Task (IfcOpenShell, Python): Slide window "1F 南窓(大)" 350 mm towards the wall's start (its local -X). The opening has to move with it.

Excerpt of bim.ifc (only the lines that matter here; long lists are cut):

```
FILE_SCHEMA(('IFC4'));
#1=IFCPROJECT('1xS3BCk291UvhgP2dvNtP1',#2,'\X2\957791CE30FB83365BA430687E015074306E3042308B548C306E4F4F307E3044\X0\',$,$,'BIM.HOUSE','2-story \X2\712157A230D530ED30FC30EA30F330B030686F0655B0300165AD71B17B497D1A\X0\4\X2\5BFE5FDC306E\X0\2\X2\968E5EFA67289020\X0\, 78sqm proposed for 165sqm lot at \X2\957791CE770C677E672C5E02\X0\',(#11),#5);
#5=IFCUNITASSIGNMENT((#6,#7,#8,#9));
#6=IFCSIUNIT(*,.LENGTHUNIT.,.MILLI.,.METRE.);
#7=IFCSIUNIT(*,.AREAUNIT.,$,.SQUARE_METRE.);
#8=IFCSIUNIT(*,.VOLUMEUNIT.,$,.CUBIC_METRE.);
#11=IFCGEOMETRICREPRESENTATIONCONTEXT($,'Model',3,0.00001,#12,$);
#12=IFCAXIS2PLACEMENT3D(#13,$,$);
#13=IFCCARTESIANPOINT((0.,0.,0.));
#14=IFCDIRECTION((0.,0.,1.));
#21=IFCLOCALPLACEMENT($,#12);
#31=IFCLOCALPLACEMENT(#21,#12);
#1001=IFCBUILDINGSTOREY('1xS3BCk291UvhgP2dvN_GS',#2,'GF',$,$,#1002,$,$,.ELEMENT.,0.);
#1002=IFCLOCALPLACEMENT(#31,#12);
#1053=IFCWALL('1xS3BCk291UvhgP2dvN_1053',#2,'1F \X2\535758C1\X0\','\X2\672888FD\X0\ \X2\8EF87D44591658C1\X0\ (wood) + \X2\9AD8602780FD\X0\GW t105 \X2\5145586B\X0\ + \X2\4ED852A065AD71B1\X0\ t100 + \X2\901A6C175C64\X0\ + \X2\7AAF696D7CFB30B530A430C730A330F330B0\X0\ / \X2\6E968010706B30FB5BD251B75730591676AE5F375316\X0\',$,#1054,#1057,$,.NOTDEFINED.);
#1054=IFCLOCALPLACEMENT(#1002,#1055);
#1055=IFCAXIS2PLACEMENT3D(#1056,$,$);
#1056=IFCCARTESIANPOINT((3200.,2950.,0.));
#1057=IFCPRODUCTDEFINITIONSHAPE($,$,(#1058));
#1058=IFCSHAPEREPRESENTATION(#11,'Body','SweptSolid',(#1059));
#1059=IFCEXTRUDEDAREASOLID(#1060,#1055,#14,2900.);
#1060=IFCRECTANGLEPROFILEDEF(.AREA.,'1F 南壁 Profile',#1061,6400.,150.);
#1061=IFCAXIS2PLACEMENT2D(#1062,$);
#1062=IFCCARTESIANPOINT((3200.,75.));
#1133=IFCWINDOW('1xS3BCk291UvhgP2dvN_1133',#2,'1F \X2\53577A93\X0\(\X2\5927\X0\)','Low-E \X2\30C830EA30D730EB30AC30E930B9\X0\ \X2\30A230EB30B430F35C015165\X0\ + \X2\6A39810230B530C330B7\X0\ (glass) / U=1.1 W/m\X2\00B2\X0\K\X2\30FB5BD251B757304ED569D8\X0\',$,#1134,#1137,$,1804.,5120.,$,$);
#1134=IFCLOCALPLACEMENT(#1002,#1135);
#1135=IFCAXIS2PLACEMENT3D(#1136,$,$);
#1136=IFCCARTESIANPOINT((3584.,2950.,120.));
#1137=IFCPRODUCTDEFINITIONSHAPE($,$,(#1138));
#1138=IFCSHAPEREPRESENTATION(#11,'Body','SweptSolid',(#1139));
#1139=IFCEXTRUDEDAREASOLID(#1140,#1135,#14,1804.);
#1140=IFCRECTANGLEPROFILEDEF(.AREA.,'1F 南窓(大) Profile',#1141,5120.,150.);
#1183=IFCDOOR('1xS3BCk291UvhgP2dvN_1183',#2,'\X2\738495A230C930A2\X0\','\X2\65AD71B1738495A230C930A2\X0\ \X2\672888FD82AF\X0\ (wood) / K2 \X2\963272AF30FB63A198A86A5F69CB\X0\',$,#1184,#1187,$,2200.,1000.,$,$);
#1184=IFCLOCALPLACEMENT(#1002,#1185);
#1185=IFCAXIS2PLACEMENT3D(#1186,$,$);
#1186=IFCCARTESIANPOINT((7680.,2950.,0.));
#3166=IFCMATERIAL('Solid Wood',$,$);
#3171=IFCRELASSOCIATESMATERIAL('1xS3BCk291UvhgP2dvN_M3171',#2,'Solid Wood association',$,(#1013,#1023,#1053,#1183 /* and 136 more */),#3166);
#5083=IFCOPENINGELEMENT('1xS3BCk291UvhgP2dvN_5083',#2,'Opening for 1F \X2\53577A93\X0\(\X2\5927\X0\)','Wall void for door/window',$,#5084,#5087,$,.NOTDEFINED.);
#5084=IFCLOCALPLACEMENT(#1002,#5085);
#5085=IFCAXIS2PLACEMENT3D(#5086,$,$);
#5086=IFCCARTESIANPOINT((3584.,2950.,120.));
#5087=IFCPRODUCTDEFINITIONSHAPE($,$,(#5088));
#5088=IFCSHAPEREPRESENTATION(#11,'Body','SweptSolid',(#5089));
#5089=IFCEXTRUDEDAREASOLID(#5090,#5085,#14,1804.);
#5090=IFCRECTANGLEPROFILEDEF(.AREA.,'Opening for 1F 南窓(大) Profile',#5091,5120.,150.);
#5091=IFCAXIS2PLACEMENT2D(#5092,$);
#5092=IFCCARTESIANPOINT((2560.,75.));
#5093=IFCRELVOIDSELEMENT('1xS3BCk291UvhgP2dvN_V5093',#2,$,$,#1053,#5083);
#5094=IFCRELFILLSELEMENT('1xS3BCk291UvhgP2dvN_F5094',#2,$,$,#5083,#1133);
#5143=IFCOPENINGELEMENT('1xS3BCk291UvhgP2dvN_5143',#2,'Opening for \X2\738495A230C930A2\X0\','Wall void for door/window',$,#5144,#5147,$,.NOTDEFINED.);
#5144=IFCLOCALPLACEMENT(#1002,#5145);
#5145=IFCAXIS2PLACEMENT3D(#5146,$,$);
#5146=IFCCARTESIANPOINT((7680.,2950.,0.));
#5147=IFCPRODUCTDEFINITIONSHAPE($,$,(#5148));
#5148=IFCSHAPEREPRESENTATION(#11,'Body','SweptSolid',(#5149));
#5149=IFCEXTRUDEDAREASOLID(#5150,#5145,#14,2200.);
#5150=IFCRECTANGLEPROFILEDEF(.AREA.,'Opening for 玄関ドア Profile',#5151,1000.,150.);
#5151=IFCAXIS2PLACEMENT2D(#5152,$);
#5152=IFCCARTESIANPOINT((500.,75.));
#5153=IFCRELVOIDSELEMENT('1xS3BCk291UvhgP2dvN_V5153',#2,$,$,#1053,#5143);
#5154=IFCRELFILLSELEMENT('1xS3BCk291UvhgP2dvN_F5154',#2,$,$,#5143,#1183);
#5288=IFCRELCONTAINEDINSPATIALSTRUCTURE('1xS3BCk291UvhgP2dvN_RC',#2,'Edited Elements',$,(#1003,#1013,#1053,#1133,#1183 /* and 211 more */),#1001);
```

```python
import ifcopenshell
import ifcopenshell.api.geometry
import ifcopenshell.util.placement
import ifcopenshell.util.unit

model = ifcopenshell.open("bim.ifc")
unit_scale = ifcopenshell.util.unit.calculate_unit_scale(model)

window = model.by_id(1133)
opening = window.FillsVoids[0].RelatingOpeningElement
wall = opening.VoidsElements[0].RelatingBuildingElement

wall_matrix = ifcopenshell.util.placement.get_local_placement(wall.ObjectPlacement)
shift = wall_matrix[:3, 0] * -0.35 / unit_scale
before = ifcopenshell.util.placement.get_local_placement(window.ObjectPlacement)[:3, 3].copy()

# The window is not placed relative to its opening, so move both.
for product in (opening, window):
    matrix = ifcopenshell.util.placement.get_local_placement(product.ObjectPlacement)
    matrix[:3, 3] += shift
    ifcopenshell.api.geometry.edit_object_placement(model, product=product, matrix=matrix, is_si=False)

after = ifcopenshell.util.placement.get_local_placement(window.ObjectPlacement)[:3, 3]
print("window moved by", (after - before).round(3) + 0.0)

model.write("bim-out.ifc")
```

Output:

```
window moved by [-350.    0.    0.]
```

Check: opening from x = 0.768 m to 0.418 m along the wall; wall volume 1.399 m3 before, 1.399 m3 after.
